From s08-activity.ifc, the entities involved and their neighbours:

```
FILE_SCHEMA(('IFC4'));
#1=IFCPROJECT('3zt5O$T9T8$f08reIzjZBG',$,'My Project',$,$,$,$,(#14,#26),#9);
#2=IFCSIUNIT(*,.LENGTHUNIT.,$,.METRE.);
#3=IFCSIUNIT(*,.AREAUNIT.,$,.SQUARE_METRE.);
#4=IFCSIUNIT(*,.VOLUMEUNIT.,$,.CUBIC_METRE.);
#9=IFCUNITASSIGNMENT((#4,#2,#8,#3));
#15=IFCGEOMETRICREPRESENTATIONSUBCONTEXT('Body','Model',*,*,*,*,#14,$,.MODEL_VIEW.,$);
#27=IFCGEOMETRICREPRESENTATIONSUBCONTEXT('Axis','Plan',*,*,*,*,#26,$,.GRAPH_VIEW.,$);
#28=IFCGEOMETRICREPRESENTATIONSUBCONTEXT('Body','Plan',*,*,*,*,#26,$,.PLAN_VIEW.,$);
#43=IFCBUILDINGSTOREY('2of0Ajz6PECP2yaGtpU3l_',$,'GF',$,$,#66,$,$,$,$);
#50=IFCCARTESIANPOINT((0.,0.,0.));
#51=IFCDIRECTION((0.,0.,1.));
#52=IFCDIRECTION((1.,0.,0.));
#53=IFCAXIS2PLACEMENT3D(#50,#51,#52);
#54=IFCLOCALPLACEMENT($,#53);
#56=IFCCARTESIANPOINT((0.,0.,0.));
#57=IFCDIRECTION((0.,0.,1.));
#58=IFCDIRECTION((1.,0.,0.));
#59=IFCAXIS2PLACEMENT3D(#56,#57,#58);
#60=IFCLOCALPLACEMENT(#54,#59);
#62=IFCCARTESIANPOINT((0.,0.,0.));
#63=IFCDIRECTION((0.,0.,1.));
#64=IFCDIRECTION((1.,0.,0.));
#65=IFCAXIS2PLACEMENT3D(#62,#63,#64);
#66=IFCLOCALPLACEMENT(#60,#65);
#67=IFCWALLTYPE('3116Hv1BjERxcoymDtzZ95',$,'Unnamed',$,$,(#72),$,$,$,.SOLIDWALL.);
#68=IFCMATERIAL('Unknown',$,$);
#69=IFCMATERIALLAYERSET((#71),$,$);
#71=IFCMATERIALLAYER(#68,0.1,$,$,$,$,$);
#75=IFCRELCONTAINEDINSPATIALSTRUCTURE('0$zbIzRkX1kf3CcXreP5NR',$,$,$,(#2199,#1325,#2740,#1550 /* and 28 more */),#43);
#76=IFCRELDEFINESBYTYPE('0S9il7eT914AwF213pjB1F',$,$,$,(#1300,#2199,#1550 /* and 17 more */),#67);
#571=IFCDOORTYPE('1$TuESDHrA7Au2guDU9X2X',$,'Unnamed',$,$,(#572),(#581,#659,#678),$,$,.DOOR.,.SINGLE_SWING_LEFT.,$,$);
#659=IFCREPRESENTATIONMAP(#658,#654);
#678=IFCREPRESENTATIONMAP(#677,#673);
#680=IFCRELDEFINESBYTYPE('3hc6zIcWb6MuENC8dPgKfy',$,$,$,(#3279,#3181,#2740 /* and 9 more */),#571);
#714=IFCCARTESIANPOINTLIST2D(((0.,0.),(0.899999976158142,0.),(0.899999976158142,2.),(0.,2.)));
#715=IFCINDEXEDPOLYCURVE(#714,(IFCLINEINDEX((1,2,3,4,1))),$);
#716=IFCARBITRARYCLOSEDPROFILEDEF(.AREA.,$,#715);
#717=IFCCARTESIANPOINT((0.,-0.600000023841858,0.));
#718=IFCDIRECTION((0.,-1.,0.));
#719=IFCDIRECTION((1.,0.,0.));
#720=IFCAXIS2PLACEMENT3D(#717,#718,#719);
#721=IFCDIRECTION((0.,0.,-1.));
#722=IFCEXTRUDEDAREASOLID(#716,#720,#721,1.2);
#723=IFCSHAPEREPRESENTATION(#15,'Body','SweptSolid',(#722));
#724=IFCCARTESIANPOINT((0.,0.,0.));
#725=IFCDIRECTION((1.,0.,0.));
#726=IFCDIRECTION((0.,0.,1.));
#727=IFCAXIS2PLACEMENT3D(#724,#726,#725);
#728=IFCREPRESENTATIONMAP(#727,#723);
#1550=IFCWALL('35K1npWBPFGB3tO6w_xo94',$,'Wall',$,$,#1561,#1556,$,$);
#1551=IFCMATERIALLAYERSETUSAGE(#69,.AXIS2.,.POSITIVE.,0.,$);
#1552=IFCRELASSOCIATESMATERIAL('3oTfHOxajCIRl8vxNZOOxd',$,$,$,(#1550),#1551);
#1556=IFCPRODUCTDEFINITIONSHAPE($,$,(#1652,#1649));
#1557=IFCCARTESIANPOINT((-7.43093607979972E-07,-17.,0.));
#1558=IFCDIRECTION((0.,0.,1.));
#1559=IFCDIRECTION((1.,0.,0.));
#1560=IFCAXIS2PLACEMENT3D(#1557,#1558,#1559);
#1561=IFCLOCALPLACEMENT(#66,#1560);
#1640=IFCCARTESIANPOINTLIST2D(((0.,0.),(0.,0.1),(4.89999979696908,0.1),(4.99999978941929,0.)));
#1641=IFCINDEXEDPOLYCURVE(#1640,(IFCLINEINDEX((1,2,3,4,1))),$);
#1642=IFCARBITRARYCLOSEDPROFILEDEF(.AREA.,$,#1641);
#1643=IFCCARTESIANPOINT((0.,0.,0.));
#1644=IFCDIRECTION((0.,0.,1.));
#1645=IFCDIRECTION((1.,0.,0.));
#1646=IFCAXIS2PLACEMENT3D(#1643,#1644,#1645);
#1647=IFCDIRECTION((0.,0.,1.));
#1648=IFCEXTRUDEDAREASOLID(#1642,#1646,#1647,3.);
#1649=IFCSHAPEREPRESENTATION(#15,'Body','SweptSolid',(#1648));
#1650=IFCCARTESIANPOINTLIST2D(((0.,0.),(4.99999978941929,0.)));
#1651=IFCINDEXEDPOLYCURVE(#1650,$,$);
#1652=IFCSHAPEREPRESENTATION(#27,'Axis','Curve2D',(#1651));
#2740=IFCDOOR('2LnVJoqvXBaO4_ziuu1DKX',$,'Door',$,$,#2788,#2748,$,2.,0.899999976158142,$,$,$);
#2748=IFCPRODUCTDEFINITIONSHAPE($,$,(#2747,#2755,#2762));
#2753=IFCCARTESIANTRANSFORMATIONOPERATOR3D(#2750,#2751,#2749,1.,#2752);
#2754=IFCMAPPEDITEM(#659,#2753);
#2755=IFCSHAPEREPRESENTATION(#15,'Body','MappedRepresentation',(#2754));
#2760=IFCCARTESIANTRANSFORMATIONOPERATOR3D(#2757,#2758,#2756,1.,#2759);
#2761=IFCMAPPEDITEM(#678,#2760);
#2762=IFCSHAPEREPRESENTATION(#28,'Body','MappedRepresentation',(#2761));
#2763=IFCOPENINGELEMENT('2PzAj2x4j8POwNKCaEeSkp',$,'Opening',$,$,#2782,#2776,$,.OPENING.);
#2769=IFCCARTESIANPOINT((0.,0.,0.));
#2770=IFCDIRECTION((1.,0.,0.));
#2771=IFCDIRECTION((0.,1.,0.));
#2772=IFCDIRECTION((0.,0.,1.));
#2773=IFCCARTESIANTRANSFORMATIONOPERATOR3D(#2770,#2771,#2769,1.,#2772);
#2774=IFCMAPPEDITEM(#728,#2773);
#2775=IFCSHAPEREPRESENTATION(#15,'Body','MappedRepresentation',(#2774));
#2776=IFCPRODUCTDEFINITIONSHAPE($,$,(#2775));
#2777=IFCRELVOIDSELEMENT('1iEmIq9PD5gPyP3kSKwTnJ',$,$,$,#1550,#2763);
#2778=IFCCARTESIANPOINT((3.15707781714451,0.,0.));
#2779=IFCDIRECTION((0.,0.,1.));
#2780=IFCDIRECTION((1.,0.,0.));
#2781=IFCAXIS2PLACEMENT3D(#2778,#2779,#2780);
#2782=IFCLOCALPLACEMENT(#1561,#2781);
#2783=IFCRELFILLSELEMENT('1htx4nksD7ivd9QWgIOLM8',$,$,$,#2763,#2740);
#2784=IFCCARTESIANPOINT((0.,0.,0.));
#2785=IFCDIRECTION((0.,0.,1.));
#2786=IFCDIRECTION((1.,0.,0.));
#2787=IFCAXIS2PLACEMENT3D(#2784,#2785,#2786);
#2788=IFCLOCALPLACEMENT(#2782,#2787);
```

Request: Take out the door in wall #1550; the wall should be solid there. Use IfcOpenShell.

```python
import ifcopenshell
import ifcopenshell.api.feature
import ifcopenshell.api.root
import ifcopenshell.geom
import ifcopenshell.util.shape

model = ifcopenshell.open("s08-activity.ifc")
settings = ifcopenshell.geom.settings()


def volume(element):
    """Net volume in cubic metres, openings subtracted."""
    shape = ifcopenshell.geom.create_shape(settings, element)
    return ifcopenshell.util.shape.get_volume(shape.geometry)


door = model.by_id(2740)
opening = door.FillsVoids[0].RelatingOpeningElement
wall = opening.VoidsElements[0].RelatingBuildingElement
before = volume(wall)

ifcopenshell.api.root.remove_product(model, product=door)
ifcopenshell.api.feature.remove_feature(model, feature=opening)

after = volume(wall)

print(f"wall volume {before:.3f} -> {after:.3f} m3")

model.write("s08-activity_edited.ifc")
```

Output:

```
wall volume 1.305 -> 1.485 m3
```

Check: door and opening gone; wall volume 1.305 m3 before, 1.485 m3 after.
